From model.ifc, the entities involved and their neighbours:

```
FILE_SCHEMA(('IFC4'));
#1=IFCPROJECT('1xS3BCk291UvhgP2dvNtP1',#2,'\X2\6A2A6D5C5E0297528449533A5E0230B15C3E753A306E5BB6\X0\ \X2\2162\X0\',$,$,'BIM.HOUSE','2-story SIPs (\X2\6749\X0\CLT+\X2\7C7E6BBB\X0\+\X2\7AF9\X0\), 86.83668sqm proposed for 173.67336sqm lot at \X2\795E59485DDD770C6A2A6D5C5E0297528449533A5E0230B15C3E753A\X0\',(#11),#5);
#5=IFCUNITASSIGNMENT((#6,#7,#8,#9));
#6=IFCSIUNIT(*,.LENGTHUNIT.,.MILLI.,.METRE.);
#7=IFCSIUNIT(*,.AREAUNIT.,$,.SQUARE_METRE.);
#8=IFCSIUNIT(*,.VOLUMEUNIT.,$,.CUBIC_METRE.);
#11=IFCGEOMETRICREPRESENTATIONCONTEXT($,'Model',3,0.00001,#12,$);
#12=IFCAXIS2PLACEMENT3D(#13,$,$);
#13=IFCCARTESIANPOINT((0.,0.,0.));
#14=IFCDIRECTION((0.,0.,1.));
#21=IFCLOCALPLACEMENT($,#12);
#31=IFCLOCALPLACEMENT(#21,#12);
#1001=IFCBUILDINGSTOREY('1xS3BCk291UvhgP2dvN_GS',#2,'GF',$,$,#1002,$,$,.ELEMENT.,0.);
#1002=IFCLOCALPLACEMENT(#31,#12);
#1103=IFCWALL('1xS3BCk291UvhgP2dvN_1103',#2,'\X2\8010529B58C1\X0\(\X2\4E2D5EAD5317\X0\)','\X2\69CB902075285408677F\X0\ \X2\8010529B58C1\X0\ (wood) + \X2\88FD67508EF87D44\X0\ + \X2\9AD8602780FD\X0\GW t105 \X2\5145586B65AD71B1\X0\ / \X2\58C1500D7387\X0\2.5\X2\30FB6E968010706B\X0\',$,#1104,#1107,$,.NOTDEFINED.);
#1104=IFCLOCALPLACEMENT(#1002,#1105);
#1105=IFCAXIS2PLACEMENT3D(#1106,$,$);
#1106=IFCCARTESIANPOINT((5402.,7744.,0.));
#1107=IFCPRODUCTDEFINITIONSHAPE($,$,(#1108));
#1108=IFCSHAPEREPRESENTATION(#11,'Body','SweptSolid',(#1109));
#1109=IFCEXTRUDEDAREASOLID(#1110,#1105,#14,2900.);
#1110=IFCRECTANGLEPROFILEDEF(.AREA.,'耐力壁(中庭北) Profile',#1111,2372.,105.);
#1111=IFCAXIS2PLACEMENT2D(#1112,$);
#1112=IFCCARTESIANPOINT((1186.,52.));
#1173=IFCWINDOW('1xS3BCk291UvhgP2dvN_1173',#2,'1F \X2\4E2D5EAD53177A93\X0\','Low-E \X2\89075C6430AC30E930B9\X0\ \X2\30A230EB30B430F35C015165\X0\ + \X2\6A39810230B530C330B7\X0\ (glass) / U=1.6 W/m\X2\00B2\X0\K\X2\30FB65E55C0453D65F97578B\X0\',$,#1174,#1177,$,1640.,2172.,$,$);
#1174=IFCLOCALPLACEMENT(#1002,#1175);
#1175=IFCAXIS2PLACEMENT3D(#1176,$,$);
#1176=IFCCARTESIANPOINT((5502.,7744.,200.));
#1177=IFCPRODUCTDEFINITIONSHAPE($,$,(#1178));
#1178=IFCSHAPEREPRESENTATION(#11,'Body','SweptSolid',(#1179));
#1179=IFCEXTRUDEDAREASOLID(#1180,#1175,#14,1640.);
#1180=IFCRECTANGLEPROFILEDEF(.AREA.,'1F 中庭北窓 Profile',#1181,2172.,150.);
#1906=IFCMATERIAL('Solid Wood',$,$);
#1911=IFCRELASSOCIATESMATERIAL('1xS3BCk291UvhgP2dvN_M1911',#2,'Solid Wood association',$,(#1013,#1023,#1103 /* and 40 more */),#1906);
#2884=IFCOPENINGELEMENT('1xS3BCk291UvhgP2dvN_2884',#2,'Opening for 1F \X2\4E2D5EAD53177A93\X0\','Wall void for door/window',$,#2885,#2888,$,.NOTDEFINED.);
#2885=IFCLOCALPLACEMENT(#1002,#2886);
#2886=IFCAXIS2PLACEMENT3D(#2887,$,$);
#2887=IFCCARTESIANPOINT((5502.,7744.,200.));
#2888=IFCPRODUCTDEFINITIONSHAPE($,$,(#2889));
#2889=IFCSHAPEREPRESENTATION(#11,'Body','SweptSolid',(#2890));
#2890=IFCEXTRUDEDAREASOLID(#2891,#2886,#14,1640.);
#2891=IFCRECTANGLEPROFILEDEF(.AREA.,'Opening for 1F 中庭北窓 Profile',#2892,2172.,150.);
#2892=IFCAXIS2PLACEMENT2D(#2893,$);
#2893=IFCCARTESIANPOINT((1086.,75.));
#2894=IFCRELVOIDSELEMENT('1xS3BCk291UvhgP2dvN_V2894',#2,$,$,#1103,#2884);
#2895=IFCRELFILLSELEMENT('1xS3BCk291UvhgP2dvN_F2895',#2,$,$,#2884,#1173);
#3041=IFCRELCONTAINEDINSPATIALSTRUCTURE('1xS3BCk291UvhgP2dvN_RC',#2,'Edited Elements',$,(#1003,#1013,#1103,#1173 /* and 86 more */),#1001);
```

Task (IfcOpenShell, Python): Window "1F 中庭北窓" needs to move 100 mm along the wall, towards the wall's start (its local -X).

```python
import ifcopenshell
import ifcopenshell.api.geometry
import ifcopenshell.util.placement

model = ifcopenshell.open("model.ifc")

window = model.by_guid("1xS3BCk291UvhgP2dvN_1173")
opening = window.FillsVoids[0].RelatingOpeningElement
wall = opening.VoidsElements[0].RelatingBuildingElement

wall_matrix = ifcopenshell.util.placement.get_local_placement(wall.ObjectPlacement)
shift = wall_matrix[:3, 0] * -100.0
before = ifcopenshell.util.placement.get_local_placement(window.ObjectPlacement)[:3, 3].copy()

# The window is not placed relative to its opening, so move both.
for product in (opening, window):
    matrix = ifcopenshell.util.placement.get_local_placement(product.ObjectPlacement)
    matrix[:3, 3] += shift
    ifcopenshell.api.geometry.edit_object_placement(model, product=product, matrix=matrix, is_si=False)

after = ifcopenshell.util.placement.get_local_placement(window.ObjectPlacement)[:3, 3]
print("window moved by", (after - before).round(3) + 0.0)

model.write("model-out.ifc")
```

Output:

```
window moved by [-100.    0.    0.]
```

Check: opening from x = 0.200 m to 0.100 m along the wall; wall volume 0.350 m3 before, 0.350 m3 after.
